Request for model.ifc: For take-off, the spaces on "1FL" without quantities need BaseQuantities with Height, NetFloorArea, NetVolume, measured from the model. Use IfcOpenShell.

First a look at what the model holds.

```python
import ifcopenshell
import ifcopenshell.util.element
import ifcopenshell.util.unit

model = ifcopenshell.open("model.ifc")
print(model.schema)
for unit_type in ("LENGTHUNIT", "AREAUNIT", "VOLUMEUNIT"):
    print(unit_type, ifcopenshell.util.unit.calculate_unit_scale(model, unit_type))
storey = next(s for s in model.by_type("IfcBuildingStorey") if s.Name == "1FL")
spaces = [e for e in ifcopenshell.util.element.get_decomposition(storey) if e.is_a("IfcSpace")]
for e in sorted(spaces, key=lambda e: e.id()):
    print(e.id(), e.is_a(), e.Name, list(ifcopenshell.util.element.get_psets(e, qtos_only=True)), sep=" | ")
```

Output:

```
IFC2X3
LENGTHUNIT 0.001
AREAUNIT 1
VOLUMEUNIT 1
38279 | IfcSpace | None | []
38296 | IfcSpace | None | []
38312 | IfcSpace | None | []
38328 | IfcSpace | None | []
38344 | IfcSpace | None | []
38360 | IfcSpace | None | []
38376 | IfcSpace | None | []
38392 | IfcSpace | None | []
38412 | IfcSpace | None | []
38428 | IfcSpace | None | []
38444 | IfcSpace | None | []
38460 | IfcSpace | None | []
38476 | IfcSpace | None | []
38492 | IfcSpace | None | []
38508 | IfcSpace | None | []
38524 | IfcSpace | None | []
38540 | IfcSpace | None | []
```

```python
import ifcopenshell
import ifcopenshell.api.pset
import ifcopenshell.geom
import ifcopenshell.util.element
import ifcopenshell.util.shape
import ifcopenshell.util.unit

model = ifcopenshell.open("model.ifc")
unit_scale = ifcopenshell.util.unit.calculate_unit_scale(model)
area_scale = ifcopenshell.util.unit.calculate_unit_scale(model, "AREAUNIT")
volume_scale = ifcopenshell.util.unit.calculate_unit_scale(model, "VOLUMEUNIT")
settings = ifcopenshell.geom.settings()

storey = next(s for s in model.by_type("IfcBuildingStorey") if s.Name == "1FL")
spaces = [e for e in ifcopenshell.util.element.get_decomposition(storey) if e.is_a("IfcSpace")]

for e in sorted(spaces, key=lambda e: e.id()):
    if ifcopenshell.util.element.get_psets(e, qtos_only=True, should_inherit=False):
        continue
    # Geometry comes back in metres, in the element's own axes.
    shape = ifcopenshell.geom.create_shape(settings, e)
    values = {
        "Height": ifcopenshell.util.shape.get_z(shape.geometry) / unit_scale,
        "NetFloorArea": ifcopenshell.util.shape.get_footprint_area(shape.geometry) / area_scale,
        "NetVolume": ifcopenshell.util.shape.get_volume(shape.geometry) / volume_scale,
    }
    qto = ifcopenshell.api.pset.add_qto(model, product=e, name="BaseQuantities")
    ifcopenshell.api.pset.edit_qto(model, qto=qto, properties=values)
    print(e.id(), {k: round(v, 3) for k, v in values.items()})

model.write("model_updated.ifc")
```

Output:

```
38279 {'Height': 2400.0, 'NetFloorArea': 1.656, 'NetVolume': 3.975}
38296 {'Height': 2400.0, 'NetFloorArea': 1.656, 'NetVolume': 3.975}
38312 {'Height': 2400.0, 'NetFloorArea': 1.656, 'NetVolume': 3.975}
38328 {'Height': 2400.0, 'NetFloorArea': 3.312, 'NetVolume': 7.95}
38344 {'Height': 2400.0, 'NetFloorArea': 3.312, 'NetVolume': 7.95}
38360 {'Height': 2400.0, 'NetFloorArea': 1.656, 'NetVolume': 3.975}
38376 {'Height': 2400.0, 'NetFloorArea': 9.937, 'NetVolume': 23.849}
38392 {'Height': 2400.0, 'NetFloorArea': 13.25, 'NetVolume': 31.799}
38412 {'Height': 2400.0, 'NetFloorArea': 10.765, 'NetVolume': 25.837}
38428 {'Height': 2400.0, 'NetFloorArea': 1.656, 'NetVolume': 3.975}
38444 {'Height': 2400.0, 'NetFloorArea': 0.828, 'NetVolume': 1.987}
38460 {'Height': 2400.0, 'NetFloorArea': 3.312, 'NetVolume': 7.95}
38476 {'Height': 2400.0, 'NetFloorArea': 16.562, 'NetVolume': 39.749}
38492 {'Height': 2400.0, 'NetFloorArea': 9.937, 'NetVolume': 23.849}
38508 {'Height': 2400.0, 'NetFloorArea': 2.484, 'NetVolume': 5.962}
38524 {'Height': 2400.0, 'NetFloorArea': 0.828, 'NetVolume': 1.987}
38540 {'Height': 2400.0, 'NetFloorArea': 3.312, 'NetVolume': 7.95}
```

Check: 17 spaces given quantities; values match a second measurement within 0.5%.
